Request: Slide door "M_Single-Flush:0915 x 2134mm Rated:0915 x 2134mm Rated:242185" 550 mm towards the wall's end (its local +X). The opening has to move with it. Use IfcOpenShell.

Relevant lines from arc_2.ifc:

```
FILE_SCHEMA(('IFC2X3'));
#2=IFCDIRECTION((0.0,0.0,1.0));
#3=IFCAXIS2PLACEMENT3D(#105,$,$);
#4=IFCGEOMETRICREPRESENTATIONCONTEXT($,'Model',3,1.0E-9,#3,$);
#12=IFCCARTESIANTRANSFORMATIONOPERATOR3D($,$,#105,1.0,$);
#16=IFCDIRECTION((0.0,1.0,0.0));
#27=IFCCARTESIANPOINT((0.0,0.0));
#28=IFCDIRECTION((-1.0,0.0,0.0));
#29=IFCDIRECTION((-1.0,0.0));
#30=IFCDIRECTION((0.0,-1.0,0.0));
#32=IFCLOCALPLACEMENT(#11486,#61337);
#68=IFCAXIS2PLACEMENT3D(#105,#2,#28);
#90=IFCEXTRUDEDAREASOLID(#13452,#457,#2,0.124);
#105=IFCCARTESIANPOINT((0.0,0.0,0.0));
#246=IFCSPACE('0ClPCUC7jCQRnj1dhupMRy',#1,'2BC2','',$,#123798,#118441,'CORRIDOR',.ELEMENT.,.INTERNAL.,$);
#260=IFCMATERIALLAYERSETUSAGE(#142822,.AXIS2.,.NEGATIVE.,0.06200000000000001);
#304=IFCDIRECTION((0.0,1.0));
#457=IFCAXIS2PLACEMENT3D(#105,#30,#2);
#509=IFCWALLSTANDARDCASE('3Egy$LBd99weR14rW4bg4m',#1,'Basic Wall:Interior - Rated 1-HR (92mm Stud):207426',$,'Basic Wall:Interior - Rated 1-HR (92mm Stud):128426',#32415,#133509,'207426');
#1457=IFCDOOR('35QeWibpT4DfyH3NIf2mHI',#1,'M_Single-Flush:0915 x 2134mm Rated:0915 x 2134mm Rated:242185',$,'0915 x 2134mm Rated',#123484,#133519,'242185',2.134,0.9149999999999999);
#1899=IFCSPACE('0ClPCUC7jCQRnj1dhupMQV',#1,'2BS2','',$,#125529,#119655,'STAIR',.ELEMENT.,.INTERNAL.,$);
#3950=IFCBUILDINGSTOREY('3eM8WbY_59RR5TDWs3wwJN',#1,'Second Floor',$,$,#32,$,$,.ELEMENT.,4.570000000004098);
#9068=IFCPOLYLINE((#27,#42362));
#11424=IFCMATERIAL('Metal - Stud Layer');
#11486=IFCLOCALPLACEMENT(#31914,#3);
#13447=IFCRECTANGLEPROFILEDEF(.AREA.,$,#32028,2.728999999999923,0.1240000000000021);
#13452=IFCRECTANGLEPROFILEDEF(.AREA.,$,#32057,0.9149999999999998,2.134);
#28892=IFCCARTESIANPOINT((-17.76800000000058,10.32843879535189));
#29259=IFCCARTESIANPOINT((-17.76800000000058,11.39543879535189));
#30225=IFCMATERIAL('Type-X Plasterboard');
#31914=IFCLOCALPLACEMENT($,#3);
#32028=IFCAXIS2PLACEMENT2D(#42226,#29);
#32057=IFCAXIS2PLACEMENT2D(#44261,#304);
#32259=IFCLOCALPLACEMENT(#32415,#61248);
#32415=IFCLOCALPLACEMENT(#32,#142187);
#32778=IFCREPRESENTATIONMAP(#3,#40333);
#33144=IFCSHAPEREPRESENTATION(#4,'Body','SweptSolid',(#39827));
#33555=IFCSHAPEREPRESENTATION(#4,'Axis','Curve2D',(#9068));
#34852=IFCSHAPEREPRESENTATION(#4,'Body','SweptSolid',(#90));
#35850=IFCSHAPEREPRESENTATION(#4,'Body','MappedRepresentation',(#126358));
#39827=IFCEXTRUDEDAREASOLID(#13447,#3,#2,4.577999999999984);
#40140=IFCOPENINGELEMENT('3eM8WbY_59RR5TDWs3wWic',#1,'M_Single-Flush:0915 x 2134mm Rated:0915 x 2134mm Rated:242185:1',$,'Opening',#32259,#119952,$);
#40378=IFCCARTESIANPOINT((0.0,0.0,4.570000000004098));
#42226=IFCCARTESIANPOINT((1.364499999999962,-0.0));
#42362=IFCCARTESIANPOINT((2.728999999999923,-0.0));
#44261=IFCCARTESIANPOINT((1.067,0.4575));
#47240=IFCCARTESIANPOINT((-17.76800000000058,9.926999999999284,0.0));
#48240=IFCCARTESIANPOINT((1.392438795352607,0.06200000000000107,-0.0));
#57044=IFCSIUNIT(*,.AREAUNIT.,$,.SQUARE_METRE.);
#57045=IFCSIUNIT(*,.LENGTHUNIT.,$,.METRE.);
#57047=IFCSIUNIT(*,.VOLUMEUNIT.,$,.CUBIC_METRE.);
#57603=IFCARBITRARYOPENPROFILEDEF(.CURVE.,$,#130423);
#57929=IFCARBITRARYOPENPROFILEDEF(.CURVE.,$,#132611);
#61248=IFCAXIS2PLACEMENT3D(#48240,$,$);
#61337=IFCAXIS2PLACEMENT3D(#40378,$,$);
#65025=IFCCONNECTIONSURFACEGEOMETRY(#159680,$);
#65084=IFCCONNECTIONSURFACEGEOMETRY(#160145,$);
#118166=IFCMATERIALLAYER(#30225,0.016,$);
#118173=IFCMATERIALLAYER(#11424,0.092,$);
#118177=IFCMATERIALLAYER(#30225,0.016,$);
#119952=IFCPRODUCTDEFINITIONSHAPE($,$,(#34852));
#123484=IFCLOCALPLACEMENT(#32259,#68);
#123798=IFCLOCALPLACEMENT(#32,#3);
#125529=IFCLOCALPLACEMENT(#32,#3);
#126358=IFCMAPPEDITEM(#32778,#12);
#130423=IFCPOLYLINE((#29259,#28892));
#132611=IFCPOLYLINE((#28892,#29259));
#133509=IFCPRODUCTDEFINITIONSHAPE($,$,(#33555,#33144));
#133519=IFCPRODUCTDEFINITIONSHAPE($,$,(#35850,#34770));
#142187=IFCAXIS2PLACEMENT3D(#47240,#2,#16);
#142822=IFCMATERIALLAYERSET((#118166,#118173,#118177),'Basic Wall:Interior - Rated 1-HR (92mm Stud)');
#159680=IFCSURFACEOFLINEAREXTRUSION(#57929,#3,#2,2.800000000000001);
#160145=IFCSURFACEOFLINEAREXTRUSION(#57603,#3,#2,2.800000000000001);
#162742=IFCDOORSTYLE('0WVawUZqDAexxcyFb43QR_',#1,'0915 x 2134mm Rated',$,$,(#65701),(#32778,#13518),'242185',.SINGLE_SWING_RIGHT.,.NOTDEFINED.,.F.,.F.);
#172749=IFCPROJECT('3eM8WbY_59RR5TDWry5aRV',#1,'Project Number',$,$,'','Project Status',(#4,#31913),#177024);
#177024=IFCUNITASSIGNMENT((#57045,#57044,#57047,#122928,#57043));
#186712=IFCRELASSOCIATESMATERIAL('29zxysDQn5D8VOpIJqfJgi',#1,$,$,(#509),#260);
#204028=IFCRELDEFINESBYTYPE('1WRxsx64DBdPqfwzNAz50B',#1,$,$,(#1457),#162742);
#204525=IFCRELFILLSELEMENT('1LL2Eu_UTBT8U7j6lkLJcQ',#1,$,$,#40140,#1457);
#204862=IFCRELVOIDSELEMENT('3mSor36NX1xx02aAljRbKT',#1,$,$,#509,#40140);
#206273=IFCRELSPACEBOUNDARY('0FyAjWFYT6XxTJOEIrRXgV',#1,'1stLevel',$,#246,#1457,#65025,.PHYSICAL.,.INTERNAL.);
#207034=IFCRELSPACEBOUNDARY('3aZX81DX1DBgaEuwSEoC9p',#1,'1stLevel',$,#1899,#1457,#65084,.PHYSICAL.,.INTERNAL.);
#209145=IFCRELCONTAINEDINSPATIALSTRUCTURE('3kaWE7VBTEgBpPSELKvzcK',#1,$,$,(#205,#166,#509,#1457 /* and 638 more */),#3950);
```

```python
import numpy as np
import ifcopenshell
import ifcopenshell.api.geometry
import ifcopenshell.util.placement

model = ifcopenshell.open("arc_2.ifc")

door = model.by_guid("35QeWibpT4DfyH3NIf2mHI")
opening = door.FillsVoids[0].RelatingOpeningElement
wall = opening.VoidsElements[0].RelatingBuildingElement

wall_matrix = ifcopenshell.util.placement.get_local_placement(wall.ObjectPlacement)
shift = wall_matrix[:3, 0] * 0.55
before = ifcopenshell.util.placement.get_local_placement(door.ObjectPlacement)[:3, 3].copy()

# The door is placed relative to its opening, so it follows when the opening moves.
matrix = ifcopenshell.util.placement.get_local_placement(opening.ObjectPlacement)
matrix[:3, 3] += shift
ifcopenshell.api.geometry.edit_object_placement(
    model, product=opening, matrix=matrix, is_si=False, should_transform_children=True
)

# Space boundary surfaces are stored in each space's coordinates; move them too.
for rel in door.ProvidesBoundaries:
    if not rel.ConnectionGeometry:
        continue
    surface = rel.ConnectionGeometry.SurfaceOnRelatingElement
    space_matrix = ifcopenshell.util.placement.get_local_placement(rel.RelatingSpace.ObjectPlacement)
    point = np.array(surface.Position.Location.Coordinates) + space_matrix[:3, :3].T @ shift
    surface.Position = model.createIfcAxis2Placement3D(
        model.createIfcCartesianPoint(point.tolist()), surface.Position.Axis, surface.Position.RefDirection
    )

after = ifcopenshell.util.placement.get_local_placement(door.ObjectPlacement)[:3, 3]
print("door moved by", (after - before).round(3) + 0.0)

model.write("arc_2_updated.ifc")
```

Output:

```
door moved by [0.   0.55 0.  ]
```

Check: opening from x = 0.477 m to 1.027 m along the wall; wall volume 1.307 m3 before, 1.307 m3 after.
